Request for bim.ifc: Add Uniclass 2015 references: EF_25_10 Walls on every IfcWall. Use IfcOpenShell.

First a look at what the model holds.

```python
import ifcopenshell

model = ifcopenshell.open("bim.ifc")
print(model.schema)
print("classifications:", [c.Name for c in model.by_type("IfcClassification")])
for ifc_class in ("IfcDoor", "IfcRoof", "IfcStair", "IfcWall", "IfcWindow"):
    print(ifc_class, len(model.by_type(ifc_class)))
```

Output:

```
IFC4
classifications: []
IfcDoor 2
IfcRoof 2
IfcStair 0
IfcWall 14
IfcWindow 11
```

```python
import ifcopenshell
import ifcopenshell.api.classification

model = ifcopenshell.open("bim.ifc")

system = ifcopenshell.api.classification.add_classification(model, classification="Uniclass 2015")

codes = {
    "IfcWall": ("EF_25_10", "Walls"),
}
for ifc_class, (code, name) in codes.items():
    products = model.by_type(ifc_class)
    ifcopenshell.api.classification.add_reference(
        model, products=products, classification=system, identification=code, name=name
    )
    print(code, len(products))

model.write("bim_rev.ifc")
```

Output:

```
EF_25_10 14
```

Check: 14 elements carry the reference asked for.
